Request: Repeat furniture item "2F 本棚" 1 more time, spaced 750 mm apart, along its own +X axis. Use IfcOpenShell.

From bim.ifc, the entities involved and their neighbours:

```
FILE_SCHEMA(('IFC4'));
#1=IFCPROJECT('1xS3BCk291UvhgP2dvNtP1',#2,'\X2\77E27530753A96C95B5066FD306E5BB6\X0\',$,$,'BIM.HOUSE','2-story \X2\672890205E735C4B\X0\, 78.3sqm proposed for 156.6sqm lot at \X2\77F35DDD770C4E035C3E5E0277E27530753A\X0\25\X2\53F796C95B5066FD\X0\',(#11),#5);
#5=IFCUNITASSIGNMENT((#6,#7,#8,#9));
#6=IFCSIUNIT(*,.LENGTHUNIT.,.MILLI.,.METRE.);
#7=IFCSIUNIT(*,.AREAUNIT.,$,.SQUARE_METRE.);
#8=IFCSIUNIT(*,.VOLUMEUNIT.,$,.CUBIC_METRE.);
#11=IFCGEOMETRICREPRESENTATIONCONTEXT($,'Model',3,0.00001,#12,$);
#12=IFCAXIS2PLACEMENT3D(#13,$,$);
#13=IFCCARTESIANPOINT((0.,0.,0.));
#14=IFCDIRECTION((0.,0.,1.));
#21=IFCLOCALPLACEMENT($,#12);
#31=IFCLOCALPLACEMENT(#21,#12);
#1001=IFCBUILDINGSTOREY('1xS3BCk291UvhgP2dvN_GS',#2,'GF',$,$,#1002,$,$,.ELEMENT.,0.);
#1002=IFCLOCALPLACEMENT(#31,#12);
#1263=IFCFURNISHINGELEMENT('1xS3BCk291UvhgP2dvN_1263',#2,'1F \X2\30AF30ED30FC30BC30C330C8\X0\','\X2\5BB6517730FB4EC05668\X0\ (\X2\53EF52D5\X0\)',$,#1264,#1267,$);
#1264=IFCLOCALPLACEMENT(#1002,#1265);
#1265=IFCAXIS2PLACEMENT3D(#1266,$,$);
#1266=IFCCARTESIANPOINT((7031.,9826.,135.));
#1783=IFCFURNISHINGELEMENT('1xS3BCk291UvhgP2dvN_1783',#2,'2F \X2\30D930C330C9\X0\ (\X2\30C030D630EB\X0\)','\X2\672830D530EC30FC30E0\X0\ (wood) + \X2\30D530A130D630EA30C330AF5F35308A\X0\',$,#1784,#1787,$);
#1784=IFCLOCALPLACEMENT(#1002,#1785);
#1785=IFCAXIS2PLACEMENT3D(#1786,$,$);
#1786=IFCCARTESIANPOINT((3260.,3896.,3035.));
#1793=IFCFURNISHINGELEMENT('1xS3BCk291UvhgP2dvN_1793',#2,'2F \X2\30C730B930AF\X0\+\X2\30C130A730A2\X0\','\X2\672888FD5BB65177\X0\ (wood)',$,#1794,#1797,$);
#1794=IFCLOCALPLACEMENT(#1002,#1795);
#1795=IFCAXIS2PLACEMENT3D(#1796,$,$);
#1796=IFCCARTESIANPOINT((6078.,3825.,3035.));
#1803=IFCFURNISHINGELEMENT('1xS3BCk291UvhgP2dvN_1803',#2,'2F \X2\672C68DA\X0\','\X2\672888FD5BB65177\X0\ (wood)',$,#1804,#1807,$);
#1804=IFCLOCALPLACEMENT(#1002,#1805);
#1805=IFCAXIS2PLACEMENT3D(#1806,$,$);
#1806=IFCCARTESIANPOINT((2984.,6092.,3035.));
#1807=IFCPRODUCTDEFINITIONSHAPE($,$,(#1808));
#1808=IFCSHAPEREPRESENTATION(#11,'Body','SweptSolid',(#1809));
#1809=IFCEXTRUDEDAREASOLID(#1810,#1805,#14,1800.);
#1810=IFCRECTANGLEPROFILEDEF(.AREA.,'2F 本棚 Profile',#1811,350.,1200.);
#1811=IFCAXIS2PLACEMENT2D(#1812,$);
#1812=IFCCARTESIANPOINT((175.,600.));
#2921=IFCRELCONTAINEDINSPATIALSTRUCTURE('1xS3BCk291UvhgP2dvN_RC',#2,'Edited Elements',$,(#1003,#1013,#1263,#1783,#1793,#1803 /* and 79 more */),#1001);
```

```python
import ifcopenshell
import ifcopenshell.api.geometry
import ifcopenshell.api.root
import ifcopenshell.util.element
import ifcopenshell.util.placement

model = ifcopenshell.open("bim.ifc")


def reuse_history(source, copy):
    """copy_class also copies each property set's owner history, people and application; keep the originals."""
    for rel in copy.IsDefinedBy:
        if rel.is_a("IfcRelDefinesByProperties") and (history := rel.RelatingPropertyDefinition.OwnerHistory):
            rel.RelatingPropertyDefinition.OwnerHistory = source.OwnerHistory
            ifcopenshell.util.element.remove_deep2(model, history)


source = model.by_id(1803)
base = ifcopenshell.util.placement.get_local_placement(source.ObjectPlacement)
step = base[:3, 0] * 750.0

for i in range(1, 2):
    copy = ifcopenshell.api.root.copy_class(model, product=source)
    copy.Representation = ifcopenshell.util.element.copy_deep(
        model, source.Representation, exclude=["IfcGeometricRepresentationContext", "IfcRepresentationMap"]
    )
    reuse_history(source, copy)
    matrix = base.copy()
    matrix[:3, 3] += i * step
    print("added at", matrix[:3, 3].round(3) + 0.0)
    ifcopenshell.api.geometry.edit_object_placement(model, product=copy, matrix=matrix, is_si=False)

model.write("bim_edited.ifc")
```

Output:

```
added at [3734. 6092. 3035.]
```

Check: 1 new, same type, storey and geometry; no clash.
